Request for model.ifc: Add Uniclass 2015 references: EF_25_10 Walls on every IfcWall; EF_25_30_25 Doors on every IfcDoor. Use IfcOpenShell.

First a look at what the model holds.

```python
import ifcopenshell

model = ifcopenshell.open("model.ifc")
print(model.schema)
print("classifications:", [c.Name for c in model.by_type("IfcClassification")])
for ifc_class in ("IfcDoor", "IfcRoof", "IfcStair", "IfcWall", "IfcWindow"):
    print(ifc_class, len(model.by_type(ifc_class)))
```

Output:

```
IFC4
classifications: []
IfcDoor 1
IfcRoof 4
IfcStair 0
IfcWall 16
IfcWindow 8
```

```python
import ifcopenshell
import ifcopenshell.api.classification

model = ifcopenshell.open("model.ifc")

system = ifcopenshell.api.classification.add_classification(model, classification="Uniclass 2015")

codes = {
    "IfcWall": ("EF_25_10", "Walls"),
    "IfcDoor": ("EF_25_30_25", "Doors"),
}
for ifc_class, (code, name) in codes.items():
    products = model.by_type(ifc_class)
    ifcopenshell.api.classification.add_reference(
        model, products=products, classification=system, identification=code, name=name
    )
    print(code, len(products))

model.write("model_updated.ifc")
```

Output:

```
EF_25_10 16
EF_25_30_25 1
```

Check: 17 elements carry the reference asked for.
